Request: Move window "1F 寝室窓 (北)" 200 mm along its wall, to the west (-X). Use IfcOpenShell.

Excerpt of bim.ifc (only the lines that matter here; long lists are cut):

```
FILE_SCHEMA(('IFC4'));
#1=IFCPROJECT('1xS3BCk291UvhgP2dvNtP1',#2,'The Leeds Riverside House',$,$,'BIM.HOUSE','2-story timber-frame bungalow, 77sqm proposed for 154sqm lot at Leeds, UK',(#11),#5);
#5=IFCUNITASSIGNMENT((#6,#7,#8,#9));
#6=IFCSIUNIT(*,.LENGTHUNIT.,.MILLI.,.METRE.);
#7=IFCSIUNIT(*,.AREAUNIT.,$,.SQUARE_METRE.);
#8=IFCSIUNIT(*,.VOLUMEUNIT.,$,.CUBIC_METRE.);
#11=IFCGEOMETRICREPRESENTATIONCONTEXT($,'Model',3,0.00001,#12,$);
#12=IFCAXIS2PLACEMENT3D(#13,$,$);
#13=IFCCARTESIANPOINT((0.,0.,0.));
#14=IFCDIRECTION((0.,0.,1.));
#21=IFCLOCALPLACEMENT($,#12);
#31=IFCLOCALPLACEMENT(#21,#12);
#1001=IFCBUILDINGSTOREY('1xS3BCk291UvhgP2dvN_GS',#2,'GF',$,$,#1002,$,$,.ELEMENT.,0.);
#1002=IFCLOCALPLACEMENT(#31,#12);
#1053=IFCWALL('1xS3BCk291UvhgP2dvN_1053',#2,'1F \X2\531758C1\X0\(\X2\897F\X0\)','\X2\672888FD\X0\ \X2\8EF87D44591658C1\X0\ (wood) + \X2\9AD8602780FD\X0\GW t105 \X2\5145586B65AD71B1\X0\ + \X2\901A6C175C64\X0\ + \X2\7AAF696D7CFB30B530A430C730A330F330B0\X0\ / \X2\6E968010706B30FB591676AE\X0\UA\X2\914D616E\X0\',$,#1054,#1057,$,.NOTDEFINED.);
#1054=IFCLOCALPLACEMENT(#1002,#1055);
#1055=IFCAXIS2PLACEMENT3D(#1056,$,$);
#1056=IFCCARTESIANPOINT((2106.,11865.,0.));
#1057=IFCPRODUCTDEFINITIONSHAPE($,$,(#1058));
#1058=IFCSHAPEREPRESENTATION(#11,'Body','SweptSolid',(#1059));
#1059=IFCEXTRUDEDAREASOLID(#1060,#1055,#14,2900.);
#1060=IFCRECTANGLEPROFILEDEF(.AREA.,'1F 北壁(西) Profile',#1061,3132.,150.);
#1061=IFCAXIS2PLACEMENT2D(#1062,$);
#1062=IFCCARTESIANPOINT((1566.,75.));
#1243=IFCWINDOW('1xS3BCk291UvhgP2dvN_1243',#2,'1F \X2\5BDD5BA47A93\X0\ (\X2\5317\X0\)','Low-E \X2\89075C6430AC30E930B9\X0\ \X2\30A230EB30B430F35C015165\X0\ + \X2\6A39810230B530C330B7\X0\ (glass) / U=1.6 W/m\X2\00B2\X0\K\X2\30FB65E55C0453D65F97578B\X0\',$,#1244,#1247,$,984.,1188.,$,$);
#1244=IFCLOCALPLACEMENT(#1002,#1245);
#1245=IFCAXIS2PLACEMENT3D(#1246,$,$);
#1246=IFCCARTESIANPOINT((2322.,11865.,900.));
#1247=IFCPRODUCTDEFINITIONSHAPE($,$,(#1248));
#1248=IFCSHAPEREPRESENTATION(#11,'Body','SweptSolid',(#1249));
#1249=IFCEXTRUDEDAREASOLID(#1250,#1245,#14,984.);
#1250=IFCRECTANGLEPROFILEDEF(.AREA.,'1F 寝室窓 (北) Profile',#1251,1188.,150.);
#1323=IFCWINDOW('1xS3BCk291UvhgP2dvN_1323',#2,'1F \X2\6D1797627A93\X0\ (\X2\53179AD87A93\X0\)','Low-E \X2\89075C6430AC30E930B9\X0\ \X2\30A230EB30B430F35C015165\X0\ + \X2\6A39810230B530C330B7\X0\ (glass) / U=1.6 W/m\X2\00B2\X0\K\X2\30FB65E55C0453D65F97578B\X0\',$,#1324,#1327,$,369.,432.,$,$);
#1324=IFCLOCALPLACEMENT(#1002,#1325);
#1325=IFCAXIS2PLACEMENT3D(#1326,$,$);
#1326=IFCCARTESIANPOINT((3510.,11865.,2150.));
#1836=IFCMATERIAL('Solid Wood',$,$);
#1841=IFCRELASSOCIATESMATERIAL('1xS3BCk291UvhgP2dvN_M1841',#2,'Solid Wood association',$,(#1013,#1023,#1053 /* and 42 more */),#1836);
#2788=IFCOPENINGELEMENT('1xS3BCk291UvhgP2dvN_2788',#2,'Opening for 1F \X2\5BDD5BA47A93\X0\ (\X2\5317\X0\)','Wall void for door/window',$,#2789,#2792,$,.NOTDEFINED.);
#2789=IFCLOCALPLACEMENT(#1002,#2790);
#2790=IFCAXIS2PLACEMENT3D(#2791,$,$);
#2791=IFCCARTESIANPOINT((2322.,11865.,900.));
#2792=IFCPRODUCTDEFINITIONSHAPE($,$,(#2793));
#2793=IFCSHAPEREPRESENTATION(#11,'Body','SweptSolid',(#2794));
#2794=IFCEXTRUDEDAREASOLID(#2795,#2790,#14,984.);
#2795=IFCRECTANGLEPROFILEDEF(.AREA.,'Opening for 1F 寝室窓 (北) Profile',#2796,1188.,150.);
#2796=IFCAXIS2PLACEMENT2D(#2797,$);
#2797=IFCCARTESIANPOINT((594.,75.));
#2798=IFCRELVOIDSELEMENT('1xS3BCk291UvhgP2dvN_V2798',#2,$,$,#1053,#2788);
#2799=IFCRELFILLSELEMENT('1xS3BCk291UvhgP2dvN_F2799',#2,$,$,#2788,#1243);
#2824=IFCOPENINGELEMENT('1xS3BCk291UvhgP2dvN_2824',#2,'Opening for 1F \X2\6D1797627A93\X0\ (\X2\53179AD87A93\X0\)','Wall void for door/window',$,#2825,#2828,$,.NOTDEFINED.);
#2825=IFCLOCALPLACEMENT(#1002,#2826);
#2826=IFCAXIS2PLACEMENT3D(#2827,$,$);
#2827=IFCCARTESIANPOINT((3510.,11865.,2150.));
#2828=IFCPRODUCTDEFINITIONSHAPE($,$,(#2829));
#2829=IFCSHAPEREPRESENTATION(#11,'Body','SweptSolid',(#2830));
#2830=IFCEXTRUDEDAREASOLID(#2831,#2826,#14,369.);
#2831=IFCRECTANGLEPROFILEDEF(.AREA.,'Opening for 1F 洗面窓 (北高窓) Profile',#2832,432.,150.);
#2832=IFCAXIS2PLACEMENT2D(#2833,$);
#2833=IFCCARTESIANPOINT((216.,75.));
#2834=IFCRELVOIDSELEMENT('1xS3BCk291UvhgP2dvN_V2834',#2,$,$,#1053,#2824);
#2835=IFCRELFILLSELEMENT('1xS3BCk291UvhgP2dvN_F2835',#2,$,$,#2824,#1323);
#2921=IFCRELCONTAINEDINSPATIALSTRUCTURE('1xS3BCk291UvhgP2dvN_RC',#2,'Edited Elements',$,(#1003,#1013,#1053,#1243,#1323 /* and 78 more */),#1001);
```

```python
import ifcopenshell
import ifcopenshell.api.geometry
import ifcopenshell.util.placement
import ifcopenshell.util.unit

model = ifcopenshell.open("bim.ifc")
unit_scale = ifcopenshell.util.unit.calculate_unit_scale(model)

window = model.by_guid("1xS3BCk291UvhgP2dvN_1243")
opening = window.FillsVoids[0].RelatingOpeningElement
wall = opening.VoidsElements[0].RelatingBuildingElement

wall_matrix = ifcopenshell.util.placement.get_local_placement(wall.ObjectPlacement)
shift = wall_matrix[:3, 0] * -0.2 / unit_scale
before = ifcopenshell.util.placement.get_local_placement(window.ObjectPlacement)[:3, 3].copy()

# The window is not placed relative to its opening, so move both.
for product in (opening, window):
    matrix = ifcopenshell.util.placement.get_local_placement(product.ObjectPlacement)
    matrix[:3, 3] += shift
    ifcopenshell.api.geometry.edit_object_placement(model, product=product, matrix=matrix, is_si=False)

after = ifcopenshell.util.placement.get_local_placement(window.ObjectPlacement)[:3, 3]
print("window moved by", (after - before).round(3) + 0.0)

model.write("bim_edited.ifc")
```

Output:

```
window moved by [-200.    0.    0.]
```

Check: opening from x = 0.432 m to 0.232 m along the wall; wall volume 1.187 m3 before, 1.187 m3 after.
